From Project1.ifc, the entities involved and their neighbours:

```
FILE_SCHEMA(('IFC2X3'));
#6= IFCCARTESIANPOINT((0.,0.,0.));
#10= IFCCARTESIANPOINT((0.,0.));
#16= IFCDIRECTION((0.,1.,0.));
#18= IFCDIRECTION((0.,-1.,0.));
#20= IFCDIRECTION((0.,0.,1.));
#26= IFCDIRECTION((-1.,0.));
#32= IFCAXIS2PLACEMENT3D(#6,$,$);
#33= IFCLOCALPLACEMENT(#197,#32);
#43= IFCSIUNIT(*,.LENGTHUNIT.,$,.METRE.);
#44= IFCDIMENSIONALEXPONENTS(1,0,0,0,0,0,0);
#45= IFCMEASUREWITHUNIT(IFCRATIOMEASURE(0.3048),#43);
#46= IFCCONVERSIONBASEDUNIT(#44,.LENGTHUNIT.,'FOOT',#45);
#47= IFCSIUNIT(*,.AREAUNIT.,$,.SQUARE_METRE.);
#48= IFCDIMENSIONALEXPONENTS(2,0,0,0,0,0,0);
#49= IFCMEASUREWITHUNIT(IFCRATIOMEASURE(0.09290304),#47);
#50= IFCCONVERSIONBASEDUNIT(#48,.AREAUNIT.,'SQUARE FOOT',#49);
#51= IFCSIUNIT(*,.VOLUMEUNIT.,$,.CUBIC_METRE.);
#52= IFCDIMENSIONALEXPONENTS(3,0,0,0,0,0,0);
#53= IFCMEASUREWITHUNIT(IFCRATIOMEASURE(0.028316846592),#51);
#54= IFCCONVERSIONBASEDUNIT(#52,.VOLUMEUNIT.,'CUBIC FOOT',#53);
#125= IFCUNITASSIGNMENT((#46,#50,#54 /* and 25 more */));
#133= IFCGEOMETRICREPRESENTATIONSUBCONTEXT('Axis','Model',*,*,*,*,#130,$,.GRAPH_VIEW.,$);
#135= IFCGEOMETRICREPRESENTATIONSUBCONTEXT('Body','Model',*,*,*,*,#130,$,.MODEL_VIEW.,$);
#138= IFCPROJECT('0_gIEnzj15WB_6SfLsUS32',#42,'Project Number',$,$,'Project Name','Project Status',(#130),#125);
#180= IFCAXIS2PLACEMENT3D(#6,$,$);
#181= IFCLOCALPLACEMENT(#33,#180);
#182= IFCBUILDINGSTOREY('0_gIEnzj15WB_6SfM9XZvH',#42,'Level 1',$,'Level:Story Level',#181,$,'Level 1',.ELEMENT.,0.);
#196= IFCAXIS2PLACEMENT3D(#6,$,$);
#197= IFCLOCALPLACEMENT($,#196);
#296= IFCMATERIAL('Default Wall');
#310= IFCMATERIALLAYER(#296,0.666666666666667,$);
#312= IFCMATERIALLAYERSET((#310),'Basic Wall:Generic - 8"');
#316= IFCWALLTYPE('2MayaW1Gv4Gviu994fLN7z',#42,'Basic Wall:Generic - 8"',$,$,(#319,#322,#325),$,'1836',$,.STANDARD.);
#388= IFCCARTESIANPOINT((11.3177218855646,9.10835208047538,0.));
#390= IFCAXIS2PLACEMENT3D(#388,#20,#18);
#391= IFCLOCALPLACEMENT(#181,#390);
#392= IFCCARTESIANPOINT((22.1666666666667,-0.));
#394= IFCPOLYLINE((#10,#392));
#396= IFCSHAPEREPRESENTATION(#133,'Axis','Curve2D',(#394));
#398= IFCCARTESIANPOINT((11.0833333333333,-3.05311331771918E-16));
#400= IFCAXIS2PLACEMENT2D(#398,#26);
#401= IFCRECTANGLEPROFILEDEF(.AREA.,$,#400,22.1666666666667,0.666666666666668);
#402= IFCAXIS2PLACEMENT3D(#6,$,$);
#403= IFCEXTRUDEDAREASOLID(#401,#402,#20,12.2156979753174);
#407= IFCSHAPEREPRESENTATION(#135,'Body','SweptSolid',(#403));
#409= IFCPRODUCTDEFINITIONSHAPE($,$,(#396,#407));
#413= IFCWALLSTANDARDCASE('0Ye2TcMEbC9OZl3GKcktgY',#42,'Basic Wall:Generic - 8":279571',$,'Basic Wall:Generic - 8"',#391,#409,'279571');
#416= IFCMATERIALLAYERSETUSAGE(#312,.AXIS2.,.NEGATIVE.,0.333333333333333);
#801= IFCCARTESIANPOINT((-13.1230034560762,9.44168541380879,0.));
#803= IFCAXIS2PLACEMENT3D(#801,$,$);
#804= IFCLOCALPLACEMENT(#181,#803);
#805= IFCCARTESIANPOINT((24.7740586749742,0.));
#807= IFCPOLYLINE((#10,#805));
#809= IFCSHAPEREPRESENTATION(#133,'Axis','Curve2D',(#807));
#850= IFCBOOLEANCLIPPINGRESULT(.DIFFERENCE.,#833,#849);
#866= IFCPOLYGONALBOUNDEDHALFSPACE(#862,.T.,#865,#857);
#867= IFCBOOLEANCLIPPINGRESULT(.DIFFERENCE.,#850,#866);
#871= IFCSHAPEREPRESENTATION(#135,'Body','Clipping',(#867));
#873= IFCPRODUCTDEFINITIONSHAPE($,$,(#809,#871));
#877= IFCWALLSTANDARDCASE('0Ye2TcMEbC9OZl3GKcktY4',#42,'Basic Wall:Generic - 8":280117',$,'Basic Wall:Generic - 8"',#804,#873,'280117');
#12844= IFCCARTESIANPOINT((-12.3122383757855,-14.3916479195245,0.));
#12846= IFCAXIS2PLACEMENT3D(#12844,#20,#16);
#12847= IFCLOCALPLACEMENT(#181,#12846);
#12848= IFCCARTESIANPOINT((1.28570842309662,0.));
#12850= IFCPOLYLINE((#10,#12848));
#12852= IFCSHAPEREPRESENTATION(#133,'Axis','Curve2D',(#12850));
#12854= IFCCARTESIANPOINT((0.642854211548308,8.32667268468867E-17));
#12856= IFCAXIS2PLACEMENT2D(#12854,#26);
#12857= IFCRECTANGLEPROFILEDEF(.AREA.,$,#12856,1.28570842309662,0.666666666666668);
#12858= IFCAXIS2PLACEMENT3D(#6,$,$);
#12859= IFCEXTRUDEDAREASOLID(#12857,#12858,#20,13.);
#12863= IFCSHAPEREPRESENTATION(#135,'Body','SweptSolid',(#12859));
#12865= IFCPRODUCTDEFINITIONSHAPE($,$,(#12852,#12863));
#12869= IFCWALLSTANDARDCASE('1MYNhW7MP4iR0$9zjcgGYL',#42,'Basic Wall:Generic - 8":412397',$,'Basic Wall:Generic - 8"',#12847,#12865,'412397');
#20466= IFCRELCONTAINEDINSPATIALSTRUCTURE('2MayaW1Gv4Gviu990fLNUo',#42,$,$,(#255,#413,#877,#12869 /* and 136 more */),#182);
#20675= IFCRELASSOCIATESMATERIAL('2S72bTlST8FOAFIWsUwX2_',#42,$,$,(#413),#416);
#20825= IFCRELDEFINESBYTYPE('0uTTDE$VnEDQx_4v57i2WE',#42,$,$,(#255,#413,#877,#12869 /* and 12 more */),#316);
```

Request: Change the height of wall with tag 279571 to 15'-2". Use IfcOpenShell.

```python
import ifcopenshell
import ifcopenshell.geom
import ifcopenshell.util.representation
import ifcopenshell.util.shape
import ifcopenshell.util.unit

model = ifcopenshell.open("Project1.ifc")
unit_scale = ifcopenshell.util.unit.calculate_unit_scale(model)
settings = ifcopenshell.geom.settings()


def volume(element):
    """Net volume in cubic metres, openings subtracted."""
    shape = ifcopenshell.geom.create_shape(settings, element)
    return ifcopenshell.util.shape.get_volume(shape.geometry)


wall = model.by_guid("0Ye2TcMEbC9OZl3GKcktgY")
before = volume(wall)

body = ifcopenshell.util.representation.get_representation(wall, "Model", "Body")
solid = body.Items[0]
old_height = solid.Depth
solid.Depth = 182 * 0.0254 / unit_scale
after = volume(wall)

print(f"height {old_height:g} -> {solid.Depth:g}, volume {before:.3f} -> {after:.3f} m3")

model.write("Project1_updated.ifc")
```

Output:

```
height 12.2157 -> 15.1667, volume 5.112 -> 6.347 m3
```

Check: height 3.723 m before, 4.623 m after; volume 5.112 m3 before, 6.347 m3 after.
